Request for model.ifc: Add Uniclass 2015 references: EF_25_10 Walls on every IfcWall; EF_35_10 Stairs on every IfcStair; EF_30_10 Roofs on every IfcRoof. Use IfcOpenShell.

First a look at what the model holds.

```python
import ifcopenshell

model = ifcopenshell.open("model.ifc")
print(model.schema)
print("classifications:", [c.Name for c in model.by_type("IfcClassification")])
for ifc_class in ("IfcDoor", "IfcRoof", "IfcStair", "IfcWall", "IfcWindow"):
    print(ifc_class, len(model.by_type(ifc_class)))
```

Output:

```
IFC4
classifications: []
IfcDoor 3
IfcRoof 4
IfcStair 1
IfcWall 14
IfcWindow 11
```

```python
import ifcopenshell
import ifcopenshell.api.classification

model = ifcopenshell.open("model.ifc")

system = ifcopenshell.api.classification.add_classification(model, classification="Uniclass 2015")

codes = {
    "IfcWall": ("EF_25_10", "Walls"),
    "IfcStair": ("EF_35_10", "Stairs"),
    "IfcRoof": ("EF_30_10", "Roofs"),
}
for ifc_class, (code, name) in codes.items():
    products = model.by_type(ifc_class)
    ifcopenshell.api.classification.add_reference(
        model, products=products, classification=system, identification=code, name=name
    )
    print(code, len(products))

model.write("model_updated.ifc")
```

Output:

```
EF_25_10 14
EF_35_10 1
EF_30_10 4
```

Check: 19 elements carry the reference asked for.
